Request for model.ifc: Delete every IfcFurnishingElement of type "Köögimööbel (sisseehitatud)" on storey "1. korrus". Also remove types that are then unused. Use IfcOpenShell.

First a look at what the model holds.

```python
import ifcopenshell
import ifcopenshell.util.element

model = ifcopenshell.open("model.ifc")
print(model.schema)
storey = next(s for s in model.by_type("IfcBuildingStorey") if s.Name == "1. korrus")
furniture = [e for e in ifcopenshell.util.element.get_decomposition(storey) if e.is_a("IfcFurnishingElement")]
seen = {}
for e in furniture:
    element_type = ifcopenshell.util.element.get_type(e)
    name = element_type.Name if element_type not in (None, e) else None
    seen[name] = seen.get(name, 0) + 1
for name, count in sorted(seen.items(), key=str):
    print(count, "x", name)
```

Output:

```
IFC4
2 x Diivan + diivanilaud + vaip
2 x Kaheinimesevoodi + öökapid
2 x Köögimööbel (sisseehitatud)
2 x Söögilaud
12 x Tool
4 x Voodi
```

```python
import ifcopenshell
import ifcopenshell.api.root
import ifcopenshell.util.element

model = ifcopenshell.open("model.ifc")

storey = next(s for s in model.by_type("IfcBuildingStorey") if s.Name == "1. korrus")
furniture = [e for e in ifcopenshell.util.element.get_decomposition(storey) if e.is_a("IfcFurnishingElement")]
targets = [e for e in furniture if (t := ifcopenshell.util.element.get_type(e)) not in (None, e) and t.Name == "Köögimööbel (sisseehitatud)"]
types = {ifcopenshell.util.element.get_type(e) for e in targets} - {None, *targets}

for e in targets:
    ifcopenshell.api.root.remove_product(model, product=e)
print(len(targets), "removed")

unused = [t for t in types if not ifcopenshell.util.element.get_types(t)]
for t in unused:
    ifcopenshell.api.root.remove_product(model, product=t)
print(len(unused), "unused types removed")

model.write("model-out.ifc")
```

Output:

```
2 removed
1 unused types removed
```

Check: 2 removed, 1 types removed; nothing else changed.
